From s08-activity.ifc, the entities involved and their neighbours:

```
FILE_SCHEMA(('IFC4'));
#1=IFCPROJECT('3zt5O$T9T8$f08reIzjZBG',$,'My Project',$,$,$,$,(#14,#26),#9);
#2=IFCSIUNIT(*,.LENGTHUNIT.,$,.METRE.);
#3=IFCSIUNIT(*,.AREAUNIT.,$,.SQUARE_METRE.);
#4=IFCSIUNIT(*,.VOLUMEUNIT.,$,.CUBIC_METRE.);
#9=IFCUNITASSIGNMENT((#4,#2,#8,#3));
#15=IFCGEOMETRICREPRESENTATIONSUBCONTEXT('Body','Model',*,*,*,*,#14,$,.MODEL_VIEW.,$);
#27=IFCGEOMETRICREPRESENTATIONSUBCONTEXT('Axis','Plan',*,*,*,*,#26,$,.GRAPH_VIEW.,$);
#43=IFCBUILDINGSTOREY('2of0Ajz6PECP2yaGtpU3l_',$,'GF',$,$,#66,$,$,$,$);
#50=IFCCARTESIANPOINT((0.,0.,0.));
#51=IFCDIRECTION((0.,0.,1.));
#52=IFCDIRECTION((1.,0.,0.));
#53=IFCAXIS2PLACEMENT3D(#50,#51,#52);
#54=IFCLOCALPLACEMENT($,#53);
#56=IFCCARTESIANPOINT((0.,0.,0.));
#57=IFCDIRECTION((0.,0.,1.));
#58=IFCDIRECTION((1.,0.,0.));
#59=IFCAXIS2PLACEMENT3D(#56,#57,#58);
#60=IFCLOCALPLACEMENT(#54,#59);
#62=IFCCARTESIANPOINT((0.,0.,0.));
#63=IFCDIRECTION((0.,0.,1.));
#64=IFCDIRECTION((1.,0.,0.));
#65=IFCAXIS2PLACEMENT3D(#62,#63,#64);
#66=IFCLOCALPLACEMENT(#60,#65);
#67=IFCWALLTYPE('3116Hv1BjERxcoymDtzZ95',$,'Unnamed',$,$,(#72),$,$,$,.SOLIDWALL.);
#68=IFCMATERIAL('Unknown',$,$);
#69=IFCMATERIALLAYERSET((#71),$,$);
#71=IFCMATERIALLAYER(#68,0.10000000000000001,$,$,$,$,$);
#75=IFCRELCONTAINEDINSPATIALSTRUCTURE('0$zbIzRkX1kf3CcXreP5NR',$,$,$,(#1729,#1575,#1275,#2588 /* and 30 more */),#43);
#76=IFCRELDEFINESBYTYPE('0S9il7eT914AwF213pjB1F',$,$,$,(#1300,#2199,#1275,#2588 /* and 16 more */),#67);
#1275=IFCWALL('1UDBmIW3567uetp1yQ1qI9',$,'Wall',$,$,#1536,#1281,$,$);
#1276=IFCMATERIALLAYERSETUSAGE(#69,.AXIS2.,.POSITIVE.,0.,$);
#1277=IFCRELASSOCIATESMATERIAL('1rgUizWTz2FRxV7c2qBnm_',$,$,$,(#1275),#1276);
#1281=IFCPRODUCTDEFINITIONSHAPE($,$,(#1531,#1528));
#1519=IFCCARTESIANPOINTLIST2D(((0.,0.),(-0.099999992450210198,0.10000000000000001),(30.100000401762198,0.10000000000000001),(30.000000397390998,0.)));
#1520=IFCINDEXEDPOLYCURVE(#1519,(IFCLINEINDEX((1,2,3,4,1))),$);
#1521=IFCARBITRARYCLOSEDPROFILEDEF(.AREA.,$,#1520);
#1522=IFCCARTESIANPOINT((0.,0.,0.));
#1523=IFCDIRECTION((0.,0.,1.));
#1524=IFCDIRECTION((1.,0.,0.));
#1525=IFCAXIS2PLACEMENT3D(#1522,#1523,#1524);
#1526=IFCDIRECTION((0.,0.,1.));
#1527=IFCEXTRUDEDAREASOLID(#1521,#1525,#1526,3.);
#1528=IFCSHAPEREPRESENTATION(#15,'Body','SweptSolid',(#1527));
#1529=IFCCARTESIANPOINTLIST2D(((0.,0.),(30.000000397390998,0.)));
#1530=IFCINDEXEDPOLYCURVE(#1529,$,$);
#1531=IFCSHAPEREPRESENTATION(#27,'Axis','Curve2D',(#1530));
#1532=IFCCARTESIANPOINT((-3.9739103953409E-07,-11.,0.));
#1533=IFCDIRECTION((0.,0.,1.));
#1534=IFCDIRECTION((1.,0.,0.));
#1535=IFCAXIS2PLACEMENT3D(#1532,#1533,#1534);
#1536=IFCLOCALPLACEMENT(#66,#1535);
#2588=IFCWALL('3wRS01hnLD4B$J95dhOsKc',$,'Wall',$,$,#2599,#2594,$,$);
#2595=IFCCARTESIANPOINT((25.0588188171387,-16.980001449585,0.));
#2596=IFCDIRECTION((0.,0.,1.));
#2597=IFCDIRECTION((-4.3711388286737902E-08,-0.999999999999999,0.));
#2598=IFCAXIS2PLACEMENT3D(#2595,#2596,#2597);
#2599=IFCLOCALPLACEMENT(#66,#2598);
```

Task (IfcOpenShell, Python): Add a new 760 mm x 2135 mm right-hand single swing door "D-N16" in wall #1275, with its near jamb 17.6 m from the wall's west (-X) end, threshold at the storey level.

```python
import numpy as np
import ifcopenshell
import ifcopenshell.api.feature
import ifcopenshell.api.geometry
import ifcopenshell.api.root
import ifcopenshell.api.spatial
import ifcopenshell.geom
import ifcopenshell.util.element
import ifcopenshell.util.placement
import ifcopenshell.util.representation
import ifcopenshell.util.shape
import ifcopenshell.util.unit

model = ifcopenshell.open("s08-activity.ifc")
unit_scale = ifcopenshell.util.unit.calculate_unit_scale(model)
settings = ifcopenshell.geom.settings()


def volume(element):
    """Net volume in cubic metres, openings subtracted."""
    shape = ifcopenshell.geom.create_shape(settings, element)
    return ifcopenshell.util.shape.get_volume(shape.geometry)


wall = model.by_guid("1UDBmIW3567uetp1yQ1qI9")
storey = ifcopenshell.util.element.get_container(wall, ifc_class="IfcBuildingStorey")
context = ifcopenshell.util.representation.get_context(model, "Model", "Body", "MODEL_VIEW")
before = volume(wall)

width, height, from_end, sill = 0.76, 2.135, 17.6, 0.0  # metres

# The wall runs along its own X axis, and the end named is its -X end.
wall_shape = ifcopenshell.geom.create_shape(settings, wall)
x, y, z = ifcopenshell.util.shape.get_vertices(wall_shape.geometry).T
start = x.min() + from_end
face, thickness = float(y.min()), float(y.max() - y.min())
wall_matrix = ifcopenshell.util.placement.get_local_placement(wall.ObjectPlacement)
level = ifcopenshell.util.placement.get_local_placement(storey.ObjectPlacement)[2, 3]


def in_wall(x, y):
    """Placement at x, y metres in the wall's axes, at sill height."""
    matrix = wall_matrix.copy()
    matrix[:, 3] = wall_matrix @ np.array([x / unit_scale, y / unit_scale, 0.0, 1.0])
    matrix[2, 3] = level + sill / unit_scale
    return matrix


# Opening: a box that overshoots both wall faces by 50 mm.
opening = ifcopenshell.api.root.create_entity(model, ifc_class="IfcOpeningElement", predefined_type="OPENING")
box = ifcopenshell.api.geometry.add_wall_representation(
    model, context=context, length=width, height=height, thickness=thickness + 0.1
)
ifcopenshell.api.geometry.assign_representation(model, product=opening, representation=box)
ifcopenshell.api.geometry.edit_object_placement(model, product=opening, matrix=in_wall(start, face - 0.05), is_si=False)
ifcopenshell.api.feature.add_feature(model, feature=opening, element=wall)

door = ifcopenshell.api.root.create_entity(model, ifc_class="IfcDoor", name="D-N16", predefined_type="DOOR")
door.OverallWidth, door.OverallHeight = width / unit_scale, height / unit_scale
door.OperationType = "SINGLE_SWING_RIGHT"
body = ifcopenshell.api.geometry.add_door_representation(
    model,
    context=context,
    overall_width=door.OverallWidth,
    overall_height=door.OverallHeight,
    operation_type="SINGLE_SWING_RIGHT",
    lining_properties={"LiningDepth": thickness / unit_scale, "ThresholdDepth": thickness / unit_scale},
)
ifcopenshell.api.geometry.assign_representation(model, product=door, representation=body)
ifcopenshell.api.spatial.assign_container(model, products=[door], relating_structure=storey)
ifcopenshell.api.feature.add_filling(model, opening=opening, element=door)

# The lining spans the wall, so the door starts at the wall face.
ifcopenshell.api.geometry.edit_object_placement(model, product=door, matrix=in_wall(start, face), is_si=False)

after = volume(wall)

print(f"wall volume {before:.3f} -> {after:.3f} m3")

model.write("s08-activity_v2.ifc")
```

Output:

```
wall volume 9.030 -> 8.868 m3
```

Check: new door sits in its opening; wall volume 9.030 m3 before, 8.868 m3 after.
